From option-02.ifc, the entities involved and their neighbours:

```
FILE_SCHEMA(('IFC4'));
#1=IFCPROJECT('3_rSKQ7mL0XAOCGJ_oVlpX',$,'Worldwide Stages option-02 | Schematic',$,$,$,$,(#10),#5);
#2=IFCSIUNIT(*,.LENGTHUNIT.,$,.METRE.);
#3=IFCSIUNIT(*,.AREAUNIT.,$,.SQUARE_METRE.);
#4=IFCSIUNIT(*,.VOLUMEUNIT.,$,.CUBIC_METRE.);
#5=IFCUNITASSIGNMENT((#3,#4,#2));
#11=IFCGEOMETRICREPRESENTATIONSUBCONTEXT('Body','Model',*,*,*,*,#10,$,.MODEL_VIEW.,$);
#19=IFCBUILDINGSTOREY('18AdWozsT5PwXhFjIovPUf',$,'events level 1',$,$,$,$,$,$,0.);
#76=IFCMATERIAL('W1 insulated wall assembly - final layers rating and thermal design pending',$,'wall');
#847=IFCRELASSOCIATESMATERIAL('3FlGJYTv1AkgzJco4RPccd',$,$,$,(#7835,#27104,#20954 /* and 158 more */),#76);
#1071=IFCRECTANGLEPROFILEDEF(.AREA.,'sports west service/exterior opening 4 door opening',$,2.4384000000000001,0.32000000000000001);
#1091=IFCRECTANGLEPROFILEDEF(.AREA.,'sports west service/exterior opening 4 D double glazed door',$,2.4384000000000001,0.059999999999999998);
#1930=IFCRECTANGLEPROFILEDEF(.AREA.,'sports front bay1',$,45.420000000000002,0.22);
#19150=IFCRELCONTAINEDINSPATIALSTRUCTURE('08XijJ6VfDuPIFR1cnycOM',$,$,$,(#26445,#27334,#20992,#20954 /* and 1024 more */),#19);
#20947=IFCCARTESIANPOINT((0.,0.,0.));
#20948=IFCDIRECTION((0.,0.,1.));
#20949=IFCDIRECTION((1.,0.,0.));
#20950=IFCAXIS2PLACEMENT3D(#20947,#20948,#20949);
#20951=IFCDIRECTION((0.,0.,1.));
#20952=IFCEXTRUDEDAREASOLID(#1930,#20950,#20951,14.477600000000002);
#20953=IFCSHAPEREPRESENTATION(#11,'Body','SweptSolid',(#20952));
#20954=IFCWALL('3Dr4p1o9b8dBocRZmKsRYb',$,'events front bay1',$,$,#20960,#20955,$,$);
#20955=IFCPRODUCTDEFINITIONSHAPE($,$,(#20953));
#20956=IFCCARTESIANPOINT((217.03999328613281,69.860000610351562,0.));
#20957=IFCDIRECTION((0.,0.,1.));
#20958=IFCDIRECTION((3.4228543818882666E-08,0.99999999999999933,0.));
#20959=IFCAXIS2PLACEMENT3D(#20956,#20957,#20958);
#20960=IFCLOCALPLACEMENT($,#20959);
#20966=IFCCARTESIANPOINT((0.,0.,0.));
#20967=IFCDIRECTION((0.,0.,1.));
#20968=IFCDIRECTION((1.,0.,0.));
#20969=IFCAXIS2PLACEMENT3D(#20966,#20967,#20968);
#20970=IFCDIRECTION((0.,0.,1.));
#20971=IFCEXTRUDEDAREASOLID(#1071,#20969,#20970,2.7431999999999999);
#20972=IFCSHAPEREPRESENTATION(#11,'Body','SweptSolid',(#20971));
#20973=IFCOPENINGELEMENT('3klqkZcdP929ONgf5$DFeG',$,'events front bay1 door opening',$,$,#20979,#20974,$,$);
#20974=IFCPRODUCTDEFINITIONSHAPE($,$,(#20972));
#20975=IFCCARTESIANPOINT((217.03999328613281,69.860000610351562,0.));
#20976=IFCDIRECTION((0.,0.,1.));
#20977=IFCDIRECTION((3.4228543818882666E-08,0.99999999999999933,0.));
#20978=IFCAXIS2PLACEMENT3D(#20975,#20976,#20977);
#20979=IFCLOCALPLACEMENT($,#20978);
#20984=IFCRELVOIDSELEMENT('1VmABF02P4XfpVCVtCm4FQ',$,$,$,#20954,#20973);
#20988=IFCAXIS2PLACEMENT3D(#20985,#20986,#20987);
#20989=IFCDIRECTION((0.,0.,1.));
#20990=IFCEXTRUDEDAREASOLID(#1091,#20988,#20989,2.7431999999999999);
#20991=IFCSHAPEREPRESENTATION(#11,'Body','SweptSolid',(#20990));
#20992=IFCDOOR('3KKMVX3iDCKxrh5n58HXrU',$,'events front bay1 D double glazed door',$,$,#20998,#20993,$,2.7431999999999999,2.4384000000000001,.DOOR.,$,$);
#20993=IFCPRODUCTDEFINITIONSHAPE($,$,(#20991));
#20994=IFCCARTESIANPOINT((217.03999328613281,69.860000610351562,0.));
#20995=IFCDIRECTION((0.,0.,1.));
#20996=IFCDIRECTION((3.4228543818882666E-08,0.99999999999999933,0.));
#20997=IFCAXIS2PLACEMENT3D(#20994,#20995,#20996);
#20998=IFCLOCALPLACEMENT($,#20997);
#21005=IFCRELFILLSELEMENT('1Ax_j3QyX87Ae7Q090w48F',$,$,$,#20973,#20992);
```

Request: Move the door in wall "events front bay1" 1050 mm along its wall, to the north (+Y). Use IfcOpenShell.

```python
import ifcopenshell
import ifcopenshell.api.geometry
import ifcopenshell.util.placement
import ifcopenshell.util.unit

model = ifcopenshell.open("option-02.ifc")
unit_scale = ifcopenshell.util.unit.calculate_unit_scale(model)

door = model.by_id(20992)
opening = door.FillsVoids[0].RelatingOpeningElement
wall = opening.VoidsElements[0].RelatingBuildingElement

wall_matrix = ifcopenshell.util.placement.get_local_placement(wall.ObjectPlacement)
shift = wall_matrix[:3, 0] * 1.05 / unit_scale
before = ifcopenshell.util.placement.get_local_placement(door.ObjectPlacement)[:3, 3].copy()

# The door is not placed relative to its opening, so move both.
for product in (opening, door):
    matrix = ifcopenshell.util.placement.get_local_placement(product.ObjectPlacement)
    matrix[:3, 3] += shift
    ifcopenshell.api.geometry.edit_object_placement(model, product=product, matrix=matrix, is_si=False)

after = ifcopenshell.util.placement.get_local_placement(door.ObjectPlacement)[:3, 3]
print("door moved by", (after - before).round(3) + 0.0)

model.write("option-02_edited.ifc")
```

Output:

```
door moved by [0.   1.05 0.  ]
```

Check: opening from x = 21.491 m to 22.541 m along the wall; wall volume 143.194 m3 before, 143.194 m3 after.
